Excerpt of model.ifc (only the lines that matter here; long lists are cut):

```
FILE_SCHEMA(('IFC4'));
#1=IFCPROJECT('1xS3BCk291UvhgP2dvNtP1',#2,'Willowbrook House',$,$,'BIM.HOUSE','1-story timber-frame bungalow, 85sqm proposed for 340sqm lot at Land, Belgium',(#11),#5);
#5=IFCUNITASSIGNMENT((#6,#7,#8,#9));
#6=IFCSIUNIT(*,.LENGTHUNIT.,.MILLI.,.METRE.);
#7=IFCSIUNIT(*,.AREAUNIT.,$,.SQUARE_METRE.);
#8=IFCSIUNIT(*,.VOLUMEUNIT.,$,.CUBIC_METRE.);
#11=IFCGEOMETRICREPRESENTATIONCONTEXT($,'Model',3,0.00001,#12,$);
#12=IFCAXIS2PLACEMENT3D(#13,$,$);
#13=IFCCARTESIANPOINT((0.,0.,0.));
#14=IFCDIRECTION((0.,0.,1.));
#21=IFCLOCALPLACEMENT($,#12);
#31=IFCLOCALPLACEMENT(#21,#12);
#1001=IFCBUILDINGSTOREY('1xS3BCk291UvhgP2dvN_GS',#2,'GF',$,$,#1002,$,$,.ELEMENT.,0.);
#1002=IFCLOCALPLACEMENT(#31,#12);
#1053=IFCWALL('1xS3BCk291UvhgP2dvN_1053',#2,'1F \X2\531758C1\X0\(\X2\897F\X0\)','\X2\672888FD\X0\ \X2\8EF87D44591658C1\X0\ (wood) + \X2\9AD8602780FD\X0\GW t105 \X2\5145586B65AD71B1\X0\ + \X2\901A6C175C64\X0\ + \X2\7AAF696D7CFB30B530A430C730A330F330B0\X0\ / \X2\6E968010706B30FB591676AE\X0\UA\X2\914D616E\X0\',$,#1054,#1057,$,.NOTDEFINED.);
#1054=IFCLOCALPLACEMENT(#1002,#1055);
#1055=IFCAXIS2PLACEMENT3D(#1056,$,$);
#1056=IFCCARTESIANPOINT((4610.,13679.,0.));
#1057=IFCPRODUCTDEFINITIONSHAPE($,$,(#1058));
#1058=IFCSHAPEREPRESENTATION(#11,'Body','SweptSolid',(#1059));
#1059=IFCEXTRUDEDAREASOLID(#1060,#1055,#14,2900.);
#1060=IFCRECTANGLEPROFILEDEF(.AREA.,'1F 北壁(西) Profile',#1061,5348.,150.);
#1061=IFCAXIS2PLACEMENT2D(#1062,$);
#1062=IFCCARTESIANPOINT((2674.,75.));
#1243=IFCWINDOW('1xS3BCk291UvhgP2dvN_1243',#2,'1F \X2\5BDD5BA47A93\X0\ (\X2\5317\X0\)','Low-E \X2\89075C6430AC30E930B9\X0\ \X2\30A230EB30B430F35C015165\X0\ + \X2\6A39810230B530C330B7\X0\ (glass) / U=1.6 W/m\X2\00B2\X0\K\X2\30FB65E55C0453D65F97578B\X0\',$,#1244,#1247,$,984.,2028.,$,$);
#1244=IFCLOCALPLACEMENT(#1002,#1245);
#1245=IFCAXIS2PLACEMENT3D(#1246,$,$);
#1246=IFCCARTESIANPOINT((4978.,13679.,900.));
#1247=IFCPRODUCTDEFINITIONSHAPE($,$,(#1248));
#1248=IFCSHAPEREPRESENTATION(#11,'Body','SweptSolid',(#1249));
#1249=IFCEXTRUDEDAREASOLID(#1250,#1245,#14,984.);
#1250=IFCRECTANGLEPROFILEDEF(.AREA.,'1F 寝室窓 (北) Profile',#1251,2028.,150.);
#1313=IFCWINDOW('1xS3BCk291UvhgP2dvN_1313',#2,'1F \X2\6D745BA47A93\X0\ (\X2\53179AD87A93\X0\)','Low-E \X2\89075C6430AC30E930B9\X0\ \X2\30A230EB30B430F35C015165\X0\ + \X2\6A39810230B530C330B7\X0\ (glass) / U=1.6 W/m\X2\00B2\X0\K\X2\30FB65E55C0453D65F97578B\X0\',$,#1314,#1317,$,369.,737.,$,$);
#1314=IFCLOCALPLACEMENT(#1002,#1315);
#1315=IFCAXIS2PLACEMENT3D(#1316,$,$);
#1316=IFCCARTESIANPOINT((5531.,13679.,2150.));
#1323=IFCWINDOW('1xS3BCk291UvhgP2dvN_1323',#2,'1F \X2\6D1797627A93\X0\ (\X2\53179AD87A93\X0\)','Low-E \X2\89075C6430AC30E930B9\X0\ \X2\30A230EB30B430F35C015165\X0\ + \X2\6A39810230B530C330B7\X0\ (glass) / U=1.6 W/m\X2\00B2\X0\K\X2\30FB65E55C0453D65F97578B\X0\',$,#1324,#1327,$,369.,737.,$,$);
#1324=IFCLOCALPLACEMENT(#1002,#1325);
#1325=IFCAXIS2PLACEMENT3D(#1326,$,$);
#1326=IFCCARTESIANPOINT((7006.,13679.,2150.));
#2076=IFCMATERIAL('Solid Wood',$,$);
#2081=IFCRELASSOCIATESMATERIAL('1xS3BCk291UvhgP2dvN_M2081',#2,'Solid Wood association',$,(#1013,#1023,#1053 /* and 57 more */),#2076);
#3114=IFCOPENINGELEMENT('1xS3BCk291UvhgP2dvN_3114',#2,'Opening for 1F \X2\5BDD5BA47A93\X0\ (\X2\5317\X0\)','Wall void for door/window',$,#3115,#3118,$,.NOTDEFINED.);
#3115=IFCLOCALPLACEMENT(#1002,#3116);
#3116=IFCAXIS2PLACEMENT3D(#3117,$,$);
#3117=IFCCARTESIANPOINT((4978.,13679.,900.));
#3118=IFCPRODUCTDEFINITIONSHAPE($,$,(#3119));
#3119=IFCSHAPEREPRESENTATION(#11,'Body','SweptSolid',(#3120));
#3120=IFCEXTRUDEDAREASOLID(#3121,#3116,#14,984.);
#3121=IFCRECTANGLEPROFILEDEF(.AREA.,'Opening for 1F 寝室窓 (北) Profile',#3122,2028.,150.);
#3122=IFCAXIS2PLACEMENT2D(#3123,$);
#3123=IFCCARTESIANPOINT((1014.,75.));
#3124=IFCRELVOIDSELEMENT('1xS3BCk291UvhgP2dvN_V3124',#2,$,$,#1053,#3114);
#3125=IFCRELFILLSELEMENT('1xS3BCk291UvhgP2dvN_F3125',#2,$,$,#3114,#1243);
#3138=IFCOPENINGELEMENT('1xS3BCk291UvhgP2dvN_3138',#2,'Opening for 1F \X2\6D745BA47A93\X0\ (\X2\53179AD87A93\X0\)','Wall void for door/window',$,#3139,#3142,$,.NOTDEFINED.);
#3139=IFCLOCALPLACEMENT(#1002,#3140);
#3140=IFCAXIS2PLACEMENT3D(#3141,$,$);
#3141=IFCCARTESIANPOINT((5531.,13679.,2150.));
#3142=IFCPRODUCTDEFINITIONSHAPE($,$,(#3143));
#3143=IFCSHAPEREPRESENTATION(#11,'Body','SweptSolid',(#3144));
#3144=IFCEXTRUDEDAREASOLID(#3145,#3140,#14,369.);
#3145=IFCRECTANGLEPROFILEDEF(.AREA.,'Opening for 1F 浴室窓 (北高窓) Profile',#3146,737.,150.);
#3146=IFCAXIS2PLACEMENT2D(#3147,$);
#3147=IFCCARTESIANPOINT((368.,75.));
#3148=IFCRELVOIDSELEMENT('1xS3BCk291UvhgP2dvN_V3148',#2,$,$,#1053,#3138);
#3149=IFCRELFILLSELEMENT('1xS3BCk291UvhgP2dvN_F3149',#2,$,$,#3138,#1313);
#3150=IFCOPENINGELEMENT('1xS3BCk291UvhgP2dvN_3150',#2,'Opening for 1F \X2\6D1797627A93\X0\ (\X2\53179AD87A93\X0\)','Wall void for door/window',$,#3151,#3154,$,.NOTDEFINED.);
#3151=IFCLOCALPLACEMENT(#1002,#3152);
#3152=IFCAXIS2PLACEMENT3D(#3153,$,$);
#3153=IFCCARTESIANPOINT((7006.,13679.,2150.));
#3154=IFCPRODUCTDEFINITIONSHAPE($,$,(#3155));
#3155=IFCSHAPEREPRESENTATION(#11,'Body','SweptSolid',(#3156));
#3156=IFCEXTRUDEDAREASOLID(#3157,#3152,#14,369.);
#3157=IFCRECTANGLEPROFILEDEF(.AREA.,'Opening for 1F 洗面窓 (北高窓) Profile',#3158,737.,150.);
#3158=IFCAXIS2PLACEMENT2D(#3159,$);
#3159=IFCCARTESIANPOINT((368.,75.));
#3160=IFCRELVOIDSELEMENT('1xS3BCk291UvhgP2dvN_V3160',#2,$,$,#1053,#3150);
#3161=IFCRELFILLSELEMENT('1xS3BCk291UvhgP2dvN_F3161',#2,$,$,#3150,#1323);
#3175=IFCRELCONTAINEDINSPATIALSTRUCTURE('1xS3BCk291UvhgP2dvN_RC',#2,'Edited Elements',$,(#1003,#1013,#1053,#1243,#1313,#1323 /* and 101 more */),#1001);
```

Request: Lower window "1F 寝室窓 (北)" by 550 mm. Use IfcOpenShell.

```python
import numpy as np
import ifcopenshell
import ifcopenshell.api.geometry
import ifcopenshell.util.placement
import ifcopenshell.util.unit

model = ifcopenshell.open("model.ifc")
unit_scale = ifcopenshell.util.unit.calculate_unit_scale(model)

window = model.by_guid("1xS3BCk291UvhgP2dvN_1243")
opening = window.FillsVoids[0].RelatingOpeningElement
dz = -550.0

shift = np.array([0.0, 0.0, dz])
# The window is not placed relative to its opening, so move both.
for product in (opening, window):
    matrix = ifcopenshell.util.placement.get_local_placement(product.ObjectPlacement)
    matrix[:3, 3] += shift
    ifcopenshell.api.geometry.edit_object_placement(model, product=product, matrix=matrix, is_si=False)

print(f"moved by {dz * unit_scale:+.3f} m")

model.write("model_updated.ifc")
```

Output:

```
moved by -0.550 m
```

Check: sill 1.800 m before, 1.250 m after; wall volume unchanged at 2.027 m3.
